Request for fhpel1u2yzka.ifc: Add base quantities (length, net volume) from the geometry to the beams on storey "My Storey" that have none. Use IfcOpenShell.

First a look at what the model holds.

```python
import ifcopenshell
import ifcopenshell.util.element
import ifcopenshell.util.unit

model = ifcopenshell.open("fhpel1u2yzka.ifc")
print(model.schema)
for unit_type in ("LENGTHUNIT", "AREAUNIT", "VOLUMEUNIT"):
    print(unit_type, ifcopenshell.util.unit.calculate_unit_scale(model, unit_type))
storey = next(s for s in model.by_type("IfcBuildingStorey") if s.Name == "My Storey")
beams = [e for e in ifcopenshell.util.element.get_decomposition(storey) if e.is_a("IfcBeam")]
for e in sorted(beams, key=lambda e: e.id()):
    print(e.id(), e.is_a(), e.Name, list(ifcopenshell.util.element.get_psets(e, qtos_only=True)), sep=" | ")
```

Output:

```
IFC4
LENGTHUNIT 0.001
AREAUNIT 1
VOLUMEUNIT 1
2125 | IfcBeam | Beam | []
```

```python
import ifcopenshell
import ifcopenshell.api.pset
import ifcopenshell.geom
import ifcopenshell.util.element
import ifcopenshell.util.shape
import ifcopenshell.util.unit

model = ifcopenshell.open("fhpel1u2yzka.ifc")
unit_scale = ifcopenshell.util.unit.calculate_unit_scale(model)
volume_scale = ifcopenshell.util.unit.calculate_unit_scale(model, "VOLUMEUNIT")
settings = ifcopenshell.geom.settings()

storey = next(s for s in model.by_type("IfcBuildingStorey") if s.Name == "My Storey")
beams = [e for e in ifcopenshell.util.element.get_decomposition(storey) if e.is_a("IfcBeam")]

for e in sorted(beams, key=lambda e: e.id()):
    if ifcopenshell.util.element.get_psets(e, qtos_only=True, should_inherit=False):
        continue
    # Geometry comes back in metres, in the element's own axes.
    shape = ifcopenshell.geom.create_shape(settings, e)
    values = {
        "Length": ifcopenshell.util.shape.get_max_xyz(shape.geometry) / unit_scale,
        "NetVolume": ifcopenshell.util.shape.get_volume(shape.geometry) / volume_scale,
    }
    qto = ifcopenshell.api.pset.add_qto(model, product=e, name="Qto_BeamBaseQuantities")
    ifcopenshell.api.pset.edit_qto(model, qto=qto, properties=values)
    print(e.id(), {k: round(v, 3) for k, v in values.items()})

model.write("fhpel1u2yzka_v2.ifc")
```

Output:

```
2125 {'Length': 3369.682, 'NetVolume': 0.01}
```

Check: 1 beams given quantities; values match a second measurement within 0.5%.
